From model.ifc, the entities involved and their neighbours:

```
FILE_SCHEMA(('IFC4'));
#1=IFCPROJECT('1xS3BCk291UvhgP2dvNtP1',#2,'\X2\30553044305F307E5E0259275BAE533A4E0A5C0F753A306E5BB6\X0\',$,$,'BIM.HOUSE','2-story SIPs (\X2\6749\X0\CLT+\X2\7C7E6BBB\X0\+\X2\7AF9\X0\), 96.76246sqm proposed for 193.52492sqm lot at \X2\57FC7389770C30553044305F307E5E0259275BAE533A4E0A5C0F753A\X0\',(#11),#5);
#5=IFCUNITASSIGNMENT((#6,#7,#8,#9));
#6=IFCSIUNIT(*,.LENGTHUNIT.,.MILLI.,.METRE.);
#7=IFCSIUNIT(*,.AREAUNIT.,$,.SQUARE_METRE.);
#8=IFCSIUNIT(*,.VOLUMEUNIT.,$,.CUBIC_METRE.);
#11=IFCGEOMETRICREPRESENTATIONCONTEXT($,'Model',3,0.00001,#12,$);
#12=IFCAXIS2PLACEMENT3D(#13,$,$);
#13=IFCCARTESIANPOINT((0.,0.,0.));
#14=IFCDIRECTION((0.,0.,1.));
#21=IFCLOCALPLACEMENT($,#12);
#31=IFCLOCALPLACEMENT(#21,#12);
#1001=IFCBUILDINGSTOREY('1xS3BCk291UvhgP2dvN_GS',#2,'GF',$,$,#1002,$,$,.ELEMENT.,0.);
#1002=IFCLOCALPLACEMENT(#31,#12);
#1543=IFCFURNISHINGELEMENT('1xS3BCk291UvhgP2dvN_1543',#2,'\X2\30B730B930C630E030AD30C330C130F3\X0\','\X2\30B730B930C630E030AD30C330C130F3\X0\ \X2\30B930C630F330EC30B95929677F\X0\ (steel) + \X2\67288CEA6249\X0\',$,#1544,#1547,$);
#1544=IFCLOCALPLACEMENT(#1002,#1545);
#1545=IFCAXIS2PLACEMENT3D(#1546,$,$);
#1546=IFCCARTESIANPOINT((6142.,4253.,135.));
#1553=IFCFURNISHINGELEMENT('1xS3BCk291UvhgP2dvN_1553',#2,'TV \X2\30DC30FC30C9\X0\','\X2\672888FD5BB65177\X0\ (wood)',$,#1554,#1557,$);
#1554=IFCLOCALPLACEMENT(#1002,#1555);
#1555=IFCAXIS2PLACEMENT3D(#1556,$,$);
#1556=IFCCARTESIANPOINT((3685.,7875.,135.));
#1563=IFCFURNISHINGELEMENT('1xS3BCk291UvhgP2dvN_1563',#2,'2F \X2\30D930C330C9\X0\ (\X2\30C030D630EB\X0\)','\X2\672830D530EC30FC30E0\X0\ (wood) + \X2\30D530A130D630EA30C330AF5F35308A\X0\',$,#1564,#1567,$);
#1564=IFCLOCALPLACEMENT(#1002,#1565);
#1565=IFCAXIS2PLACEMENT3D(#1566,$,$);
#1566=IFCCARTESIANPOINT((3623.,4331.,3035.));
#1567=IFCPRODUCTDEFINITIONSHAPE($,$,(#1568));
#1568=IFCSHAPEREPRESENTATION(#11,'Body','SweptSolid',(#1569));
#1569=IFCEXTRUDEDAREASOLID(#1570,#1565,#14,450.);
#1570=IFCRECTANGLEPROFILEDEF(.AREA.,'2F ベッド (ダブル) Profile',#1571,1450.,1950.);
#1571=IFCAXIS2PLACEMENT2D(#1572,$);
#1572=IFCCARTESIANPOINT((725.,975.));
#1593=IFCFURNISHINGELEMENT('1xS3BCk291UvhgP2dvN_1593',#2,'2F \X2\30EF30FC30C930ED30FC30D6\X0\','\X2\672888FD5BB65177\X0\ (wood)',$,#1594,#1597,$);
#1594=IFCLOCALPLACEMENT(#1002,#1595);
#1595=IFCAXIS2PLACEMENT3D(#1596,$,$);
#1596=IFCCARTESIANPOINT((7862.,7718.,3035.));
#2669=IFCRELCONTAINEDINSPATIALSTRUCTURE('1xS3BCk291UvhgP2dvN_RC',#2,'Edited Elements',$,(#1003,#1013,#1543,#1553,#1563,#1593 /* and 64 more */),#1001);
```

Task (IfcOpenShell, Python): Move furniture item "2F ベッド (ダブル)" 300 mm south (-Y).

```python
import ifcopenshell
import ifcopenshell.api.geometry
import ifcopenshell.util.placement
import ifcopenshell.util.unit

model = ifcopenshell.open("model.ifc")
unit_scale = ifcopenshell.util.unit.calculate_unit_scale(model)

item = model.by_id(1563)
matrix = ifcopenshell.util.placement.get_local_placement(item.ObjectPlacement)
matrix[1, 3] -= 0.3 / unit_scale
ifcopenshell.api.geometry.edit_object_placement(model, product=item, matrix=matrix, is_si=False)

print(ifcopenshell.util.placement.get_local_placement(item.ObjectPlacement).round(3) + 0.0)

model.write("model_edited.ifc")
```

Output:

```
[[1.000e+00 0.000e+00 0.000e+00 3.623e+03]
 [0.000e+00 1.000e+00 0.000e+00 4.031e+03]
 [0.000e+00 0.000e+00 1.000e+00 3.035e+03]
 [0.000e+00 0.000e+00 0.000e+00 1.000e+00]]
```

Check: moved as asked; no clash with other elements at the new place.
